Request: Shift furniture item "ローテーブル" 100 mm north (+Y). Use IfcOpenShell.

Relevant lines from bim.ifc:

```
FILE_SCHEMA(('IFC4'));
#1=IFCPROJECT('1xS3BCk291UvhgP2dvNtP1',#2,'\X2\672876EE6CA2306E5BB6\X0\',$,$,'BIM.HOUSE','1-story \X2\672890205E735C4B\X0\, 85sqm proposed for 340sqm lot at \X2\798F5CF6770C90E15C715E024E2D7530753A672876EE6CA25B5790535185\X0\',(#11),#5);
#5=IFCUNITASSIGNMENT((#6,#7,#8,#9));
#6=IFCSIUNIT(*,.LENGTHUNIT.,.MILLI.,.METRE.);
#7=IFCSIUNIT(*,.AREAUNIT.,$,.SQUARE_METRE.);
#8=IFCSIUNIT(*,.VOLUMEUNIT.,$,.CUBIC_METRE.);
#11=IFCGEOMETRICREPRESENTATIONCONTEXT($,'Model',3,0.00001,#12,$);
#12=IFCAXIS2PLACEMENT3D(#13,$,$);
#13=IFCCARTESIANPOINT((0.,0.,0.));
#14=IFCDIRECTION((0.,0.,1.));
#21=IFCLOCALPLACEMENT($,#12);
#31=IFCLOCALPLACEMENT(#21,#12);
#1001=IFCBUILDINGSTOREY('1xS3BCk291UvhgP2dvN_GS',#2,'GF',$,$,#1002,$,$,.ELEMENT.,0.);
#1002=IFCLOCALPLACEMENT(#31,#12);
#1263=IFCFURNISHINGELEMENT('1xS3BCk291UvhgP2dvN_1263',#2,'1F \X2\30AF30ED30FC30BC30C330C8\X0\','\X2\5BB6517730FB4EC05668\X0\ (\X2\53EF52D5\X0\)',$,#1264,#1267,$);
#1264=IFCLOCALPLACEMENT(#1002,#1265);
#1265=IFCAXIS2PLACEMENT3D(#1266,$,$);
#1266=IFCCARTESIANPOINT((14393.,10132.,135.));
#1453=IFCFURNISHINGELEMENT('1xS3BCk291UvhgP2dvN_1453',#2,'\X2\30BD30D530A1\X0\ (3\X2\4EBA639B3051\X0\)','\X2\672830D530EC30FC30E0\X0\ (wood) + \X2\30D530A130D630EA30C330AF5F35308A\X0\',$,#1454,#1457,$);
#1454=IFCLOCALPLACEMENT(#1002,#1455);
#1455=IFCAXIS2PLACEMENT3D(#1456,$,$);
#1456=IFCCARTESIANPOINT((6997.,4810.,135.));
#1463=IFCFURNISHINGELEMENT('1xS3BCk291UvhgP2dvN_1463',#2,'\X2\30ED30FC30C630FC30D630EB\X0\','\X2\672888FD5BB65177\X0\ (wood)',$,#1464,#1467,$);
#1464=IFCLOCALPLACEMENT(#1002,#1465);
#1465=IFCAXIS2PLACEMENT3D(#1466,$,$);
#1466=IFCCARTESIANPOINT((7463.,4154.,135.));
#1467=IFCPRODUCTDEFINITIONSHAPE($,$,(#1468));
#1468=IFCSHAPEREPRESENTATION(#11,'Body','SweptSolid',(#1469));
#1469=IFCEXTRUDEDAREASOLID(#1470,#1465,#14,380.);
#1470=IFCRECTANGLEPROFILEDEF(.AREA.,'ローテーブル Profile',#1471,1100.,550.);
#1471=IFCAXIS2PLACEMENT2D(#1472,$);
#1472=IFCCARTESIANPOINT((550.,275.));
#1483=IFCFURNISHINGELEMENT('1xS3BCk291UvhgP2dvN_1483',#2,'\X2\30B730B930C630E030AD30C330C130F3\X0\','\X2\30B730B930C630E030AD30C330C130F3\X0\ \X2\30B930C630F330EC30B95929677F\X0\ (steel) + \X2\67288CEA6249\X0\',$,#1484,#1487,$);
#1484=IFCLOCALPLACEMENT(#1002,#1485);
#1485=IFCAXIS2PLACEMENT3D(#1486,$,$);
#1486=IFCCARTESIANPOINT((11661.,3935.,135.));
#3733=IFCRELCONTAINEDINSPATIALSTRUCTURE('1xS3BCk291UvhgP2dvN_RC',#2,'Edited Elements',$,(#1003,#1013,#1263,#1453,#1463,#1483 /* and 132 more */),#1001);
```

```python
import ifcopenshell
import ifcopenshell.api.geometry
import ifcopenshell.util.placement
import ifcopenshell.util.unit

model = ifcopenshell.open("bim.ifc")
unit_scale = ifcopenshell.util.unit.calculate_unit_scale(model)

item = model.by_id(1463)
matrix = ifcopenshell.util.placement.get_local_placement(item.ObjectPlacement)
matrix[1, 3] += 0.1 / unit_scale
ifcopenshell.api.geometry.edit_object_placement(model, product=item, matrix=matrix, is_si=False)

print(ifcopenshell.util.placement.get_local_placement(item.ObjectPlacement).round(3) + 0.0)

model.write("bim_v2.ifc")
```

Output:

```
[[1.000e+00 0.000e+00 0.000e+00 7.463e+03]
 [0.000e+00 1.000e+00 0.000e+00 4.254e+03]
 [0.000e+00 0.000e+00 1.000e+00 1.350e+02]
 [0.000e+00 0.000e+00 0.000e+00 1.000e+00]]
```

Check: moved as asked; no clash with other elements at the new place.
